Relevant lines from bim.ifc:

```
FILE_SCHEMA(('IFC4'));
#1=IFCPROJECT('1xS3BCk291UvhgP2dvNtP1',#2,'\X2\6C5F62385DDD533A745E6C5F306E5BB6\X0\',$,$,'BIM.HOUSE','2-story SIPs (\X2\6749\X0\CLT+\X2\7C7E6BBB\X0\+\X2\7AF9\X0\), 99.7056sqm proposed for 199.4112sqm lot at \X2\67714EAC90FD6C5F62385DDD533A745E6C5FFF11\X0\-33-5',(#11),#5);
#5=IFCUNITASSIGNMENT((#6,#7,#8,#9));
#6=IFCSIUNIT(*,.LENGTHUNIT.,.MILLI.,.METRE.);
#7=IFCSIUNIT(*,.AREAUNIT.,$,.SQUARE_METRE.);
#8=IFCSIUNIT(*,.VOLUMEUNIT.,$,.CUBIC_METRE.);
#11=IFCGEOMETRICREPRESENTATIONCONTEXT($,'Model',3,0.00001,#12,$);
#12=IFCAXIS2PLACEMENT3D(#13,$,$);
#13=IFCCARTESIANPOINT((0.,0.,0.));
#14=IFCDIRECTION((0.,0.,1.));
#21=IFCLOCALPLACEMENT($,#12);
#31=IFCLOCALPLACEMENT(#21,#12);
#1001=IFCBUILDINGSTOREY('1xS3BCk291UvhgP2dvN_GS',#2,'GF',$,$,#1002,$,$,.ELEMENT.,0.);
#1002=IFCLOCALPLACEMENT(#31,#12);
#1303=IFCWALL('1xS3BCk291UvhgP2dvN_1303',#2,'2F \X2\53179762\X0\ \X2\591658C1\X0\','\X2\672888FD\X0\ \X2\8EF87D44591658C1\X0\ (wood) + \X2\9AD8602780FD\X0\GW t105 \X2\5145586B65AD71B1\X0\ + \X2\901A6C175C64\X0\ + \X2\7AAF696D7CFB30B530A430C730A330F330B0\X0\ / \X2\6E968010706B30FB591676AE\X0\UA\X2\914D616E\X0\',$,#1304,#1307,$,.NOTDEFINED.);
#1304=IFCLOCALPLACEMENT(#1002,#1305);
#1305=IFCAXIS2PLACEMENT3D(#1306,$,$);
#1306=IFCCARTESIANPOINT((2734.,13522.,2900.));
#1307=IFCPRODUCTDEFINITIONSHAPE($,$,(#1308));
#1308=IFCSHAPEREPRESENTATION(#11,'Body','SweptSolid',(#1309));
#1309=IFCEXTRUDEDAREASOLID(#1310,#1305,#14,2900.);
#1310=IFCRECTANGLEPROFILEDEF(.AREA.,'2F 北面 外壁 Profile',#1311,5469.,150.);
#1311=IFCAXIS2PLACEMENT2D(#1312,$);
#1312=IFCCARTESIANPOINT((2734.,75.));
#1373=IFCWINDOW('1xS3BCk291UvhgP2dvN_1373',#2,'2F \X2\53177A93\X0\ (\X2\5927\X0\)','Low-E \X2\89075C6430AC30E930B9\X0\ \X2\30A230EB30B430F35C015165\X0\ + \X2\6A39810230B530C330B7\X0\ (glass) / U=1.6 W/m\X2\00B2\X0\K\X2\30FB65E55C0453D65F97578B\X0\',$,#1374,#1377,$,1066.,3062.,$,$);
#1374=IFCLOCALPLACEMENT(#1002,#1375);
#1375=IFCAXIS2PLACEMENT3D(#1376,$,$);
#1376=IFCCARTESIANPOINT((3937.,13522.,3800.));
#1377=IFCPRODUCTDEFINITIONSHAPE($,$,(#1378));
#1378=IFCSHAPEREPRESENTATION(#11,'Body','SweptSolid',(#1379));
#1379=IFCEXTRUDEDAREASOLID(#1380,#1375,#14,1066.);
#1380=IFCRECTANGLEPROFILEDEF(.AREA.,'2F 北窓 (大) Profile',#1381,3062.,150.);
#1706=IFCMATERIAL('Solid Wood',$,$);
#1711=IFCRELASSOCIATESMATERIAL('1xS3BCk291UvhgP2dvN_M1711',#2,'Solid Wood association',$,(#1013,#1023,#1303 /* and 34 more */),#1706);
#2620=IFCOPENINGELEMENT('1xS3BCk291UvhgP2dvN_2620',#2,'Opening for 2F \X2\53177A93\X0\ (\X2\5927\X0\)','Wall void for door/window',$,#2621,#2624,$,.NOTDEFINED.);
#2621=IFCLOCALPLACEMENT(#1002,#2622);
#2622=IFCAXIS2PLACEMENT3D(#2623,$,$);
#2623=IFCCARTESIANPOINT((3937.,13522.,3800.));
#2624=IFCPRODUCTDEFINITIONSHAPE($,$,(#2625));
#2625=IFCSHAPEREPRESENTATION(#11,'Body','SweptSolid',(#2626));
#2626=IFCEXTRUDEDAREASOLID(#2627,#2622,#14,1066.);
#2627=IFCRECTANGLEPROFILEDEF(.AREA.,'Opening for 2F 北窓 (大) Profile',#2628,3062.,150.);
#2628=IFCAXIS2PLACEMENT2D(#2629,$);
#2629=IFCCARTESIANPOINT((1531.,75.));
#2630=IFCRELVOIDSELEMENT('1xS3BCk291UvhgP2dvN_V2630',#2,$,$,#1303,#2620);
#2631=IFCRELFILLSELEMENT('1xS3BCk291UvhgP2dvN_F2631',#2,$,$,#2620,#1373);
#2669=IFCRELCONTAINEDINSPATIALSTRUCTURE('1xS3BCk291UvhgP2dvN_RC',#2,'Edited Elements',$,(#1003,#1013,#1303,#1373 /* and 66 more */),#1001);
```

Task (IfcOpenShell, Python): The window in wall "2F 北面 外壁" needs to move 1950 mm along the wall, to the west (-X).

```python
import ifcopenshell
import ifcopenshell.api.geometry
import ifcopenshell.util.placement

model = ifcopenshell.open("bim.ifc")

window = model.by_guid("1xS3BCk291UvhgP2dvN_1373")
opening = window.FillsVoids[0].RelatingOpeningElement
wall = opening.VoidsElements[0].RelatingBuildingElement

wall_matrix = ifcopenshell.util.placement.get_local_placement(wall.ObjectPlacement)
shift = wall_matrix[:3, 0] * -1950.0
before = ifcopenshell.util.placement.get_local_placement(window.ObjectPlacement)[:3, 3].copy()

# The window is not placed relative to its opening, so move both.
for product in (opening, window):
    matrix = ifcopenshell.util.placement.get_local_placement(product.ObjectPlacement)
    matrix[:3, 3] += shift
    ifcopenshell.api.geometry.edit_object_placement(model, product=product, matrix=matrix, is_si=False)

after = ifcopenshell.util.placement.get_local_placement(window.ObjectPlacement)[:3, 3]
print("window moved by", (after - before).round(3) + 0.0)

model.write("bim_rev.ifc")
```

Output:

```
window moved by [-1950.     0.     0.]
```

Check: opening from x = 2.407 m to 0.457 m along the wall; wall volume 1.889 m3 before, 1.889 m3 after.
